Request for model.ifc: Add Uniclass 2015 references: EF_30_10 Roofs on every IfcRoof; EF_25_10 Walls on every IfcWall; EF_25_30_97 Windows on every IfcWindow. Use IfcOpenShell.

First a look at what the model holds.

```python
import ifcopenshell

model = ifcopenshell.open("model.ifc")
print(model.schema)
print("classifications:", [c.Name for c in model.by_type("IfcClassification")])
for ifc_class in ("IfcDoor", "IfcRoof", "IfcStair", "IfcWall", "IfcWindow"):
    print(ifc_class, len(model.by_type(ifc_class)))
```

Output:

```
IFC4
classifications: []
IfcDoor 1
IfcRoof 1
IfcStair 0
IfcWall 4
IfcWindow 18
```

```python
import ifcopenshell
import ifcopenshell.api.classification

model = ifcopenshell.open("model.ifc")

system = ifcopenshell.api.classification.add_classification(model, classification="Uniclass 2015")

codes = {
    "IfcRoof": ("EF_30_10", "Roofs"),
    "IfcWall": ("EF_25_10", "Walls"),
    "IfcWindow": ("EF_25_30_97", "Windows"),
}
for ifc_class, (code, name) in codes.items():
    products = model.by_type(ifc_class)
    ifcopenshell.api.classification.add_reference(
        model, products=products, classification=system, identification=code, name=name
    )
    print(code, len(products))

model.write("model-out.ifc")
```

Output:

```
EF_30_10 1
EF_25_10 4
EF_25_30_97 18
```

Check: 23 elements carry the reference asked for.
